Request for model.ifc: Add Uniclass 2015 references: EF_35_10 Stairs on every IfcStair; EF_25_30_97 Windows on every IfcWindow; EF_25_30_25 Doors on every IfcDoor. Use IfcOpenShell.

First a look at what the model holds.

```python
import ifcopenshell

model = ifcopenshell.open("model.ifc")
print(model.schema)
print("classifications:", [c.Name for c in model.by_type("IfcClassification")])
for ifc_class in ("IfcDoor", "IfcRoof", "IfcStair", "IfcWall", "IfcWindow"):
    print(ifc_class, len(model.by_type(ifc_class)))
```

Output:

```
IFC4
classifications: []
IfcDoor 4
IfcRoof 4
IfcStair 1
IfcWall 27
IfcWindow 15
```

```python
import ifcopenshell
import ifcopenshell.api.classification

model = ifcopenshell.open("model.ifc")

system = ifcopenshell.api.classification.add_classification(model, classification="Uniclass 2015")

codes = {
    "IfcStair": ("EF_35_10", "Stairs"),
    "IfcWindow": ("EF_25_30_97", "Windows"),
    "IfcDoor": ("EF_25_30_25", "Doors"),
}
for ifc_class, (code, name) in codes.items():
    products = model.by_type(ifc_class)
    ifcopenshell.api.classification.add_reference(
        model, products=products, classification=system, identification=code, name=name
    )
    print(code, len(products))

model.write("model-out.ifc")
```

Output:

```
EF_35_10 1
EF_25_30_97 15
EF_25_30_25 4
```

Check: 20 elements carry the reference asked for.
